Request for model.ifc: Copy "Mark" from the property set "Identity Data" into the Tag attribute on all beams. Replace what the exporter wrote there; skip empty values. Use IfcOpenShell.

First a look at what the model holds.

```python
import ifcopenshell
import ifcopenshell.util.element

model = ifcopenshell.open("model.ifc")
print(model.schema)
beams = model.by_type("IfcBeam")
print(len(beams), "beams")
for e in beams[:8]:
    source = ifcopenshell.util.element.get_pset(e, "Identity Data", "Mark")
    target = e.Tag
    print(e.id(), repr(source), repr(target), sep=" | ")
```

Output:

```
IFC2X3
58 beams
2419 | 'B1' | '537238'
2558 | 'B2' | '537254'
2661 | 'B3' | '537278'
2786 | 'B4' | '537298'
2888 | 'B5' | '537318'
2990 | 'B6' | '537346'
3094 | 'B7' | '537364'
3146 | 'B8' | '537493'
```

```python
import ifcopenshell
import ifcopenshell.util.element

model = ifcopenshell.open("model.ifc")

count = 0
for e in model.by_type("IfcBeam"):
    value = ifcopenshell.util.element.get_pset(e, "Identity Data", "Mark")
    current = e.Tag
    if not value or not value.strip() or current == value:
        continue
    e.Tag = value
    count += 1

print(count, "beams updated")

model.write("model_updated.ifc")
```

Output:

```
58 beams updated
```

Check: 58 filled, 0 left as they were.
